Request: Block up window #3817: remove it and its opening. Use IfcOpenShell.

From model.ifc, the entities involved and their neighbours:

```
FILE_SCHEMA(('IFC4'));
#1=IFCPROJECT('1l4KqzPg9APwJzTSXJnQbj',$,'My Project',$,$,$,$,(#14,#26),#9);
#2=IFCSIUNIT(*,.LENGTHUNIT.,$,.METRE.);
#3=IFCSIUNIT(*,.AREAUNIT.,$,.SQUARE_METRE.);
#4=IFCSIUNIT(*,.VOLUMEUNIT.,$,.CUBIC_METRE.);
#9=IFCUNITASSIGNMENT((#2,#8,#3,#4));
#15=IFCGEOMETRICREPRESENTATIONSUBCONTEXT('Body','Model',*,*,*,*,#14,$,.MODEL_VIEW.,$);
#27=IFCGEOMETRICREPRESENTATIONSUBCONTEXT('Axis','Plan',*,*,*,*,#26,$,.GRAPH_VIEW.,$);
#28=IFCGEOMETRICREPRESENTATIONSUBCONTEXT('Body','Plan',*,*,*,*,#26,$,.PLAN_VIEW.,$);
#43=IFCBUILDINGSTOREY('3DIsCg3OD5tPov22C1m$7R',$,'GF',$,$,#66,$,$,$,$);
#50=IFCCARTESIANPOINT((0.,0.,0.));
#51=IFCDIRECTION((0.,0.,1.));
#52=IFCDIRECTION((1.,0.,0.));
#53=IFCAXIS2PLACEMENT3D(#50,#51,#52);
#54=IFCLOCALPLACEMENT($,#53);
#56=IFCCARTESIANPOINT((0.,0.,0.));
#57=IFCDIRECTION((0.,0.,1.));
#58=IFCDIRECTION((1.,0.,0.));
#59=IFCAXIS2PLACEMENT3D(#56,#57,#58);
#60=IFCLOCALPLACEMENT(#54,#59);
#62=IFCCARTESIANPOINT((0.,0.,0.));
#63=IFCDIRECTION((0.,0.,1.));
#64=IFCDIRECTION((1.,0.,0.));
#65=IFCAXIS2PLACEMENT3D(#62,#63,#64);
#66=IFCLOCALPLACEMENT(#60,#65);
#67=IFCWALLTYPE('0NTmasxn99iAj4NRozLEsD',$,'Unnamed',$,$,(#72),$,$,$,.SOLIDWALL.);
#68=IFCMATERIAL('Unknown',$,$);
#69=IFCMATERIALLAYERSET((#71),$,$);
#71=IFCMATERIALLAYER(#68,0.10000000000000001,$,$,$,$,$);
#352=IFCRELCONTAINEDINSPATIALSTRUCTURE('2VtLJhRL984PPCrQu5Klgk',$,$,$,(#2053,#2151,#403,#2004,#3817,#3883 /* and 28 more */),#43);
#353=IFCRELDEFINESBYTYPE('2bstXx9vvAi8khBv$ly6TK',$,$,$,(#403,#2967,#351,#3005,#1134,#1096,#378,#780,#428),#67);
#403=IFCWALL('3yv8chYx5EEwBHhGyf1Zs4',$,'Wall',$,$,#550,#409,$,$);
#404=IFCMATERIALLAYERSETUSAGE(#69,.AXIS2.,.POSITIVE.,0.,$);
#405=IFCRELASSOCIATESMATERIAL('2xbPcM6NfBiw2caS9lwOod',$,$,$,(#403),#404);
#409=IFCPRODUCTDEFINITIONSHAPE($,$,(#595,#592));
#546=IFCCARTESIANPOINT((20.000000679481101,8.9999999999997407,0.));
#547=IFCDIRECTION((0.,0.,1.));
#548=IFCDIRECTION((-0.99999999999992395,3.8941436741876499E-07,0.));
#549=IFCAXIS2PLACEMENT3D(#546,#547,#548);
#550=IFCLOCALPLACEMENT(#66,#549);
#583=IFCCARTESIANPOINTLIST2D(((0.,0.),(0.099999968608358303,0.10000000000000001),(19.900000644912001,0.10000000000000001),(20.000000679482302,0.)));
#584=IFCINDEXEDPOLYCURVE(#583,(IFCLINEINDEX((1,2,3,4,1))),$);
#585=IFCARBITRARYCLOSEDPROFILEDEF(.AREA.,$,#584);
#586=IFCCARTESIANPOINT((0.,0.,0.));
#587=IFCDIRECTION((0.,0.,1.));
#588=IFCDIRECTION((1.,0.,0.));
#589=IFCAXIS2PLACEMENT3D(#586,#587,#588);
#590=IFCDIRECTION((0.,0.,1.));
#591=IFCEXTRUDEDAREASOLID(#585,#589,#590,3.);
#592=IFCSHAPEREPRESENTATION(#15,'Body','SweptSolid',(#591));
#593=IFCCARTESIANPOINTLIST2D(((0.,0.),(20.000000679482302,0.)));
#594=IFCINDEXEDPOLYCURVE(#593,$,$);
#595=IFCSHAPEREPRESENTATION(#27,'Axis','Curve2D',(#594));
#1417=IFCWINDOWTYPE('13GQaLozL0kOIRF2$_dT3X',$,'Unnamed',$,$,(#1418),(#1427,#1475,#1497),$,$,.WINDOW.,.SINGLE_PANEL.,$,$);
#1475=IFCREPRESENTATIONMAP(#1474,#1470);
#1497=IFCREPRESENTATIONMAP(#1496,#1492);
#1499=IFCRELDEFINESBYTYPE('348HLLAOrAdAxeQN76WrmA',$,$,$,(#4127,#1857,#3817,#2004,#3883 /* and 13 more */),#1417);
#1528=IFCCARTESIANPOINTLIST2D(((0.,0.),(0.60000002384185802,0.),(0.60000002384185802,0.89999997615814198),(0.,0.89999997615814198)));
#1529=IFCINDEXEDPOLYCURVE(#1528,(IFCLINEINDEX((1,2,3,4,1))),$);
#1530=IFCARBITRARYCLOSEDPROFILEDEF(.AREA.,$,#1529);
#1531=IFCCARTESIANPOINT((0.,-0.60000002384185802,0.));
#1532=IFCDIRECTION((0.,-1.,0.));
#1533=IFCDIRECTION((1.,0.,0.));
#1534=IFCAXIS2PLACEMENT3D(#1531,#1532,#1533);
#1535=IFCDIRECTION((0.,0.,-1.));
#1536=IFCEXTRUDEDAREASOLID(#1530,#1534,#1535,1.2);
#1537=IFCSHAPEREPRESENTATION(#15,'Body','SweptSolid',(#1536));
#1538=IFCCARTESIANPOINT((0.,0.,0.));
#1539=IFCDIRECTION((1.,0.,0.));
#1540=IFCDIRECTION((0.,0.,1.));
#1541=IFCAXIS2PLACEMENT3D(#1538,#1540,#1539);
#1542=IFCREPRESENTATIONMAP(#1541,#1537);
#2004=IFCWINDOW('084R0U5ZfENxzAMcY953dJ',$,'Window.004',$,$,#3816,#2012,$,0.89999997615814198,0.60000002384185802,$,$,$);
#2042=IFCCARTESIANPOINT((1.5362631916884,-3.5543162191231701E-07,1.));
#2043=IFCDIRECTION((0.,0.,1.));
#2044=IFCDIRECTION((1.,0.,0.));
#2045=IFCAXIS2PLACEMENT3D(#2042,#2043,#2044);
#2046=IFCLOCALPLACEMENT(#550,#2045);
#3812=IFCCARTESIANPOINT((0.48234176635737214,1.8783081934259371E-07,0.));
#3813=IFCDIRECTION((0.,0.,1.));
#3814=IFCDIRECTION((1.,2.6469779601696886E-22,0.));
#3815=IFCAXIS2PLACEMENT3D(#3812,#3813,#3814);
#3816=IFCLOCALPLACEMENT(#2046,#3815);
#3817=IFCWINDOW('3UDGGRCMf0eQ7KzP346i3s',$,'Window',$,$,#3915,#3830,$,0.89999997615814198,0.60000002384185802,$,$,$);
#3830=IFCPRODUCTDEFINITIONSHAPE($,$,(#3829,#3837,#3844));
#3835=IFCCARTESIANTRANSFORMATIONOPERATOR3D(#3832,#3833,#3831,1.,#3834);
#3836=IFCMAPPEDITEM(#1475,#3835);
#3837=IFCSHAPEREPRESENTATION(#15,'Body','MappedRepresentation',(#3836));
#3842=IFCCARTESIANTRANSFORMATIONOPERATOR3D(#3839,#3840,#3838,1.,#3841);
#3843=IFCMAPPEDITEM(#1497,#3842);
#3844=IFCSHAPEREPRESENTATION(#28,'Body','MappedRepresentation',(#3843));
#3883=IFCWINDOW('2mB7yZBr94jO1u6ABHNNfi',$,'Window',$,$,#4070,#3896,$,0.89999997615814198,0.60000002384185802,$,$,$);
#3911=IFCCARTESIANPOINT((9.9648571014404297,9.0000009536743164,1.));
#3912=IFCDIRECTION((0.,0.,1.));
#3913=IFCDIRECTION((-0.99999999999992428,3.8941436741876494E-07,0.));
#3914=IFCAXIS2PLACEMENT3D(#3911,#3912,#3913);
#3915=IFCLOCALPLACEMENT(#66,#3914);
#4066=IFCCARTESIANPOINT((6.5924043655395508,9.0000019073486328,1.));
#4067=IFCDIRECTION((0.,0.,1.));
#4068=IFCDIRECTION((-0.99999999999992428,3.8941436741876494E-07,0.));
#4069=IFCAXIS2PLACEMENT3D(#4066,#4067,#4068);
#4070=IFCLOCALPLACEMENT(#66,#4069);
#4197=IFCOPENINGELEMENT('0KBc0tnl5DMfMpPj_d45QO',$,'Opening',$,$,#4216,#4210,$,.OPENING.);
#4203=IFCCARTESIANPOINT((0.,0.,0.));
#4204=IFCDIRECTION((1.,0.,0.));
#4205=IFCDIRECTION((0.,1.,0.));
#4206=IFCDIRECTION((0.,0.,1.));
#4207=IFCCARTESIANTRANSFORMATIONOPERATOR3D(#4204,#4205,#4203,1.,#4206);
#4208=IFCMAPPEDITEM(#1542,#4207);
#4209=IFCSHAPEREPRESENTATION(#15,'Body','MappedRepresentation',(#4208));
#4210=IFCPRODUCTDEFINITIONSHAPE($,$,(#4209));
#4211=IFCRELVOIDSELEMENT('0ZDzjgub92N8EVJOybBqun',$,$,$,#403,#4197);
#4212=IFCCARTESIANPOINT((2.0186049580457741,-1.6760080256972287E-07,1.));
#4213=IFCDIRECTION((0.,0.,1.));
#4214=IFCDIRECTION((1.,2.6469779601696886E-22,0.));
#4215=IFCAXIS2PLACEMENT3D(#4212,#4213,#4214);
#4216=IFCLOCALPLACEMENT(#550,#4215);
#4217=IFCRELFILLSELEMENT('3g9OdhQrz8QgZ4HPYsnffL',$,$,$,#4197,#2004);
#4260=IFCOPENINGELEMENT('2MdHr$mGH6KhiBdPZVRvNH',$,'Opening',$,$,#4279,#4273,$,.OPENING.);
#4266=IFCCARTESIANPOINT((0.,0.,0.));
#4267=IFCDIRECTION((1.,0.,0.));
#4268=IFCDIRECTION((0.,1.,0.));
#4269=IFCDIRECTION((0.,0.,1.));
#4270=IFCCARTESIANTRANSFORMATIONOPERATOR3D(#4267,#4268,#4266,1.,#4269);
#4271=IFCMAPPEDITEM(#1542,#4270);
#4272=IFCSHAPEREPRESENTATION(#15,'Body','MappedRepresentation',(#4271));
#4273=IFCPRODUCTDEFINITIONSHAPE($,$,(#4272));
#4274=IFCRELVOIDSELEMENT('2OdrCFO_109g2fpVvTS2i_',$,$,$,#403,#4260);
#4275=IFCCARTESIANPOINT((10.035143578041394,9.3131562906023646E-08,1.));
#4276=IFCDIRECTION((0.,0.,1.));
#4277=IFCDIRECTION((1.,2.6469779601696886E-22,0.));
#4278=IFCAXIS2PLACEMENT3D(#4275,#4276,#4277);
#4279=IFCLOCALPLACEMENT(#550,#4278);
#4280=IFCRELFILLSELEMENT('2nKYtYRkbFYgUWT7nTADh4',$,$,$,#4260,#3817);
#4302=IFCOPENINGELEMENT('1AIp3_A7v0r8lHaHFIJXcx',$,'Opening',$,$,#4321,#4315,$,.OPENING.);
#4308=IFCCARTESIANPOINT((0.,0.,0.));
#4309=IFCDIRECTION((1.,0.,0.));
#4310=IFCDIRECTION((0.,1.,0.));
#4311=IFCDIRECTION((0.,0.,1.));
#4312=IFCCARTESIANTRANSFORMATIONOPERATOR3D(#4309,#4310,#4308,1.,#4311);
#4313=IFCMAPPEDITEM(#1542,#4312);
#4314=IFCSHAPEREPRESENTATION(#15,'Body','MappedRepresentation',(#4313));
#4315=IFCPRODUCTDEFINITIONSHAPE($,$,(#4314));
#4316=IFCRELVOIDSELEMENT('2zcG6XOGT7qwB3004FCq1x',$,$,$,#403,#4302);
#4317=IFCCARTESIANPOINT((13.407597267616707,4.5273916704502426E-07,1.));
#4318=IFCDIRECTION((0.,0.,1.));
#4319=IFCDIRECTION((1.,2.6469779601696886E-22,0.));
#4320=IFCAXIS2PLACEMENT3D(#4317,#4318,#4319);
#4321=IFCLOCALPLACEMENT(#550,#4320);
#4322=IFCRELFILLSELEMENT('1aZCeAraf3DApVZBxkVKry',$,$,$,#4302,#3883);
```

```python
import ifcopenshell
import ifcopenshell.api.feature
import ifcopenshell.api.root
import ifcopenshell.geom
import ifcopenshell.util.shape

model = ifcopenshell.open("model.ifc")
settings = ifcopenshell.geom.settings()


def volume(element):
    """Net volume in cubic metres, openings subtracted."""
    shape = ifcopenshell.geom.create_shape(settings, element)
    return ifcopenshell.util.shape.get_volume(shape.geometry)


window = model.by_guid("3UDGGRCMf0eQ7KzP346i3s")
opening = window.FillsVoids[0].RelatingOpeningElement
wall = opening.VoidsElements[0].RelatingBuildingElement
before = volume(wall)

ifcopenshell.api.root.remove_product(model, product=window)
ifcopenshell.api.feature.remove_feature(model, feature=opening)

after = volume(wall)

print(f"wall volume {before:.3f} -> {after:.3f} m3")

model.write("model_rev.ifc")
```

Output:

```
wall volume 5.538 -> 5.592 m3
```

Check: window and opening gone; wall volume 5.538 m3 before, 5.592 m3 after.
